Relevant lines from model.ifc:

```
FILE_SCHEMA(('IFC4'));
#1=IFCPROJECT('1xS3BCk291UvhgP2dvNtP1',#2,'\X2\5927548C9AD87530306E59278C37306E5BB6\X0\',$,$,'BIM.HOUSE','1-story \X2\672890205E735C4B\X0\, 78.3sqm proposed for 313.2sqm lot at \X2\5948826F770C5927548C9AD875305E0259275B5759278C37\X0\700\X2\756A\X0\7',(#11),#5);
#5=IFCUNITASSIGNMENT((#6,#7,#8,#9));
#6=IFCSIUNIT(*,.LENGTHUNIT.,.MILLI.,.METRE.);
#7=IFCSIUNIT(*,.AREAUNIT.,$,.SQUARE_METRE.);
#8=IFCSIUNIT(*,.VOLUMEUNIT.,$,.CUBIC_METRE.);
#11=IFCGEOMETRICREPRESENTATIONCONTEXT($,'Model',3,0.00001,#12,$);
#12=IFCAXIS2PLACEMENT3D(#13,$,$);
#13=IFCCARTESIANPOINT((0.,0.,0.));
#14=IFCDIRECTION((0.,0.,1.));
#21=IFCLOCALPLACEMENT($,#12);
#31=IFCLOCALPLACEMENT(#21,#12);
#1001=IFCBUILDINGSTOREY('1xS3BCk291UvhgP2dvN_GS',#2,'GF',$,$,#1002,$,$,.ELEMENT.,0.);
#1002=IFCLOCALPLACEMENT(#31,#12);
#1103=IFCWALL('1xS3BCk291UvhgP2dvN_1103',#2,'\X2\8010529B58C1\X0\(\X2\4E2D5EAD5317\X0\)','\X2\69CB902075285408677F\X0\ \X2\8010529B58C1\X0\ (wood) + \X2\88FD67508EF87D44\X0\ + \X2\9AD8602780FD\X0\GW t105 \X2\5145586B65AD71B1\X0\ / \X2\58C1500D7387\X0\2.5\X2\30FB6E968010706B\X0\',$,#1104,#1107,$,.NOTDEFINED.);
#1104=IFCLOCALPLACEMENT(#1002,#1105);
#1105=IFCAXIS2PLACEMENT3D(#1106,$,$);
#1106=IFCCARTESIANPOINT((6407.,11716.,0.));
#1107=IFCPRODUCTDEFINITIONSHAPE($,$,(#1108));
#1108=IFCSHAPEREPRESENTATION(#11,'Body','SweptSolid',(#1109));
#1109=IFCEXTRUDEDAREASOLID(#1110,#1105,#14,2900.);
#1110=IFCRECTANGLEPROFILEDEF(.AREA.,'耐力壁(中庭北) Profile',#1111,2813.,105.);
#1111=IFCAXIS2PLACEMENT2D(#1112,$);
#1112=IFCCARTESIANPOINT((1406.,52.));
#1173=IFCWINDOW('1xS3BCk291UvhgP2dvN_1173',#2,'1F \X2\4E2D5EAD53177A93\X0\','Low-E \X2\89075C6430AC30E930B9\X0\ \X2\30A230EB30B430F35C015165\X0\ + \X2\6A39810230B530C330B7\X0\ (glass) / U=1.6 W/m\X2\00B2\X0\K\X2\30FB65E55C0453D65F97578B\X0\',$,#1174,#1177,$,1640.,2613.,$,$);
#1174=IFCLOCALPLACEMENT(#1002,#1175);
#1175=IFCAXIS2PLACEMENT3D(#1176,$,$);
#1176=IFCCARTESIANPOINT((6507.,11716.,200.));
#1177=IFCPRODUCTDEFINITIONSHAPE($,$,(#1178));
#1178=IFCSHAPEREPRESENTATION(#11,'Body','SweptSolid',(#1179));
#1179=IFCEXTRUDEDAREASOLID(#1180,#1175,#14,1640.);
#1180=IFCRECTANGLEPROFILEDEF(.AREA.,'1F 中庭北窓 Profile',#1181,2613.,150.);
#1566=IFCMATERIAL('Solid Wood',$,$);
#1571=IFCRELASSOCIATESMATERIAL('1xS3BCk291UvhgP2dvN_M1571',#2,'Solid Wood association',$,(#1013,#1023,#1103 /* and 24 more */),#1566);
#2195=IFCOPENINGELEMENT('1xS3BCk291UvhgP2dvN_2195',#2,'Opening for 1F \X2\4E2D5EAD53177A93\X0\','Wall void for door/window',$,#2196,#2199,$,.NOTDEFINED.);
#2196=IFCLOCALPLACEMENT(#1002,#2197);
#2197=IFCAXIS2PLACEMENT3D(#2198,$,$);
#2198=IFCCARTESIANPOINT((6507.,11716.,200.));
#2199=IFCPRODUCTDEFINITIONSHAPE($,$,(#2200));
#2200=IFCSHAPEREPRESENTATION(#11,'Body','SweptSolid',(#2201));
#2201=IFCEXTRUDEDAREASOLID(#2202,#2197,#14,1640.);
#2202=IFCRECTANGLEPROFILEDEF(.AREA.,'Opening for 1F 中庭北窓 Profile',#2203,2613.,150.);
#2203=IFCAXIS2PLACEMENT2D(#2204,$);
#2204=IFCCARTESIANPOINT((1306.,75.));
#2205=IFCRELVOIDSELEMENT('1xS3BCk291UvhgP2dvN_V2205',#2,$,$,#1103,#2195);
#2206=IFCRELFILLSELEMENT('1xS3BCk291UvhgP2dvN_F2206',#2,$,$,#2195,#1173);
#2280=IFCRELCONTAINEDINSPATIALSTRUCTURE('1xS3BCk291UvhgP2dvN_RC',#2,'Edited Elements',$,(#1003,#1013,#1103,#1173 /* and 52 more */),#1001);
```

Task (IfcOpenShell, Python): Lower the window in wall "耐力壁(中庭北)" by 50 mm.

```python
import numpy as np
import ifcopenshell
import ifcopenshell.api.geometry
import ifcopenshell.util.placement
import ifcopenshell.util.unit

model = ifcopenshell.open("model.ifc")
unit_scale = ifcopenshell.util.unit.calculate_unit_scale(model)

window = model.by_guid("1xS3BCk291UvhgP2dvN_1173")
opening = window.FillsVoids[0].RelatingOpeningElement
dz = -50.0

shift = np.array([0.0, 0.0, dz])
# The window is not placed relative to its opening, so move both.
for product in (opening, window):
    matrix = ifcopenshell.util.placement.get_local_placement(product.ObjectPlacement)
    matrix[:3, 3] += shift
    ifcopenshell.api.geometry.edit_object_placement(model, product=product, matrix=matrix, is_si=False)

print(f"moved by {dz * unit_scale:+.3f} m")

model.write("model_v2.ifc")
```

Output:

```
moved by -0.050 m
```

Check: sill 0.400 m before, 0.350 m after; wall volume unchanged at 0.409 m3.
